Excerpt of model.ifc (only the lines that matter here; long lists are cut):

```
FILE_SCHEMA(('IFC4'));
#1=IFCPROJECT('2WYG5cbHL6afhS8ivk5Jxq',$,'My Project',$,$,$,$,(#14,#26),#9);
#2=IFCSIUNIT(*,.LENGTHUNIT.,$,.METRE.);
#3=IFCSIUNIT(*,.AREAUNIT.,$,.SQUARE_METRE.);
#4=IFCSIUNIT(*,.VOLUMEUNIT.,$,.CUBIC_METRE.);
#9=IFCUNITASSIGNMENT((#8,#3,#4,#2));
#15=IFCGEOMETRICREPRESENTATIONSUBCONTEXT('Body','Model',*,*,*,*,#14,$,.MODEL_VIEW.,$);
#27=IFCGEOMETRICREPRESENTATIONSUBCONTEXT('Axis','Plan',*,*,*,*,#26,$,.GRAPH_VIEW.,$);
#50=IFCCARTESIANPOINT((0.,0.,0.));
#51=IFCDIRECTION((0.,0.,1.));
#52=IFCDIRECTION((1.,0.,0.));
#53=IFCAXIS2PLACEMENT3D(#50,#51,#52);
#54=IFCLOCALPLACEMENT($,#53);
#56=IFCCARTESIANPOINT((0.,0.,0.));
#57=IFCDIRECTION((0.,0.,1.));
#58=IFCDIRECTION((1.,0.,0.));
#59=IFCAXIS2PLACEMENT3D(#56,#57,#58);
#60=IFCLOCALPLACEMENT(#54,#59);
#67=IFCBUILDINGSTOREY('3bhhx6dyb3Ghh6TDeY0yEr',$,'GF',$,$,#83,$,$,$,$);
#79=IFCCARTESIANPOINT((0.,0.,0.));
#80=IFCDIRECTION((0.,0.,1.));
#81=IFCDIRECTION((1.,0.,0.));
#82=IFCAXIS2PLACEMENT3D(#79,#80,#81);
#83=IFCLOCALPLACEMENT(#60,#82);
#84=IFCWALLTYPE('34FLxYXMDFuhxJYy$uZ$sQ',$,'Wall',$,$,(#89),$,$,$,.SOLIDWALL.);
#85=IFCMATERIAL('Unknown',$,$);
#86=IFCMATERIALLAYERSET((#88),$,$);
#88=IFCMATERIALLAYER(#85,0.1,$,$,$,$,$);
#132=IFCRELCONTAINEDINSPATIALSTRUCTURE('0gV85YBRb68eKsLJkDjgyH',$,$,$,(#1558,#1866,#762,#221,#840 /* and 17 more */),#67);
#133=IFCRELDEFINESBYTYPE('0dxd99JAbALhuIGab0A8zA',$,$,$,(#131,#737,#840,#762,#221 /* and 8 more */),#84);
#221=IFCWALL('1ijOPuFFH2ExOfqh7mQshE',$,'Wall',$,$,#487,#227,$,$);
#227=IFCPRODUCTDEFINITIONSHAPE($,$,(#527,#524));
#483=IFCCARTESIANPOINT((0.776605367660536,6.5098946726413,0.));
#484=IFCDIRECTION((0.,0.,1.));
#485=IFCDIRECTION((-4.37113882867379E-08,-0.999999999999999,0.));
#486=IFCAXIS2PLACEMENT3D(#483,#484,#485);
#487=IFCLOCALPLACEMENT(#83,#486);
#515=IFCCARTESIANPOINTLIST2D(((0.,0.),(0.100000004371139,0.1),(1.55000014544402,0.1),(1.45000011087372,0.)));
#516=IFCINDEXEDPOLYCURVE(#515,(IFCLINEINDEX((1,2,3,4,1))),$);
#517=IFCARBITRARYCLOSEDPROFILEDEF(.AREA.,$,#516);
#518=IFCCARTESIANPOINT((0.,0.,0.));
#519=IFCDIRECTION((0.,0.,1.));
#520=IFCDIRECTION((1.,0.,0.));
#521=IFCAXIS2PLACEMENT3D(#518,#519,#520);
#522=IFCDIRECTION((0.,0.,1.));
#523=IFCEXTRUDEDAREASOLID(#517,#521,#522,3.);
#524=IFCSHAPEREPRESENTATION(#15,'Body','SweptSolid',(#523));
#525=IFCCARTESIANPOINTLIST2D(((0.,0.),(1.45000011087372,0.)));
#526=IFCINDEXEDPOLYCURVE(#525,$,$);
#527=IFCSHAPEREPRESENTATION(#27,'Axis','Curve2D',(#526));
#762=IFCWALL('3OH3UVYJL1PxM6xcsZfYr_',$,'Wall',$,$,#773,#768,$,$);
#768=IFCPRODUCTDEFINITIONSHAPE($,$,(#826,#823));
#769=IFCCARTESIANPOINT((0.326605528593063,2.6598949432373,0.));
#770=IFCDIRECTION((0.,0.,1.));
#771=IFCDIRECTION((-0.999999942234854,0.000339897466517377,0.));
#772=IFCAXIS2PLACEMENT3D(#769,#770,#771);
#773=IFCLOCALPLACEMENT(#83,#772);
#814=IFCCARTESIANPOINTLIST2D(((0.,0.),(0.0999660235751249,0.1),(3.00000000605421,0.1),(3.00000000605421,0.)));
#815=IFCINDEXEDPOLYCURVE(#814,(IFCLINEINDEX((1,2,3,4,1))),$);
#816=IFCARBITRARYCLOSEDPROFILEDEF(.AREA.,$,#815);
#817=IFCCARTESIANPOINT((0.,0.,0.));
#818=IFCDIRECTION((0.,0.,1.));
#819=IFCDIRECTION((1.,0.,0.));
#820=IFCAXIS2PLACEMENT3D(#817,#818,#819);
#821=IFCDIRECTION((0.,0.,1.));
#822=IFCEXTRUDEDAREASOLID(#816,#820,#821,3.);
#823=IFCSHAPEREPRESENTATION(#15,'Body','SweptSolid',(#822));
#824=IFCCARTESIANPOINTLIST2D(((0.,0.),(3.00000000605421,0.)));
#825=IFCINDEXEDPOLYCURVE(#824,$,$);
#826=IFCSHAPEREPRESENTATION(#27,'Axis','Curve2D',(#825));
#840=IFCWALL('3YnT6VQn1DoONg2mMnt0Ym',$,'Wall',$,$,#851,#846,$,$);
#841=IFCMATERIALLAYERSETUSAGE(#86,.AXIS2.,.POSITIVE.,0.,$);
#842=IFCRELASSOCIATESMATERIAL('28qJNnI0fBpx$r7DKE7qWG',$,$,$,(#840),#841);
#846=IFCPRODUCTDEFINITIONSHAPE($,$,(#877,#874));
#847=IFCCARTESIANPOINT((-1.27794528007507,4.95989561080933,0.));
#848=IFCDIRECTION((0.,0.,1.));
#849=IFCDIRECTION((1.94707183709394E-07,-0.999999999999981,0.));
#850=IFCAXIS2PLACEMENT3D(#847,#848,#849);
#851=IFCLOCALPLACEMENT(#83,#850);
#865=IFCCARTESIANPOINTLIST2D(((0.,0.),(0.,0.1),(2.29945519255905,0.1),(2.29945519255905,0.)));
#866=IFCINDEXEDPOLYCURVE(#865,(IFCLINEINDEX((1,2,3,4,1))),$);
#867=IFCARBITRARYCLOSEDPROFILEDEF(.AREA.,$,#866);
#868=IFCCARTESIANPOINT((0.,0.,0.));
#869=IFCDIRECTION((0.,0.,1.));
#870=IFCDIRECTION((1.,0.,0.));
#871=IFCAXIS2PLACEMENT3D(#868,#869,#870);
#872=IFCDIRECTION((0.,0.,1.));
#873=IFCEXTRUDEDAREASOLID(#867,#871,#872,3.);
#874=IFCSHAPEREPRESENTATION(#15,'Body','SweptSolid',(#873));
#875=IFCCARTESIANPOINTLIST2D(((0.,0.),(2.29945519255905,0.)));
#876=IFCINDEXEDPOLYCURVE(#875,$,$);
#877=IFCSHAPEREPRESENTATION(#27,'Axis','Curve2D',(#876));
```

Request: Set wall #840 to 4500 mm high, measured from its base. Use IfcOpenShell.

```python
import ifcopenshell
import ifcopenshell.geom
import ifcopenshell.util.representation
import ifcopenshell.util.shape
import ifcopenshell.util.unit

model = ifcopenshell.open("model.ifc")
unit_scale = ifcopenshell.util.unit.calculate_unit_scale(model)
settings = ifcopenshell.geom.settings()


def volume(element):
    """Net volume in cubic metres, openings subtracted."""
    shape = ifcopenshell.geom.create_shape(settings, element)
    return ifcopenshell.util.shape.get_volume(shape.geometry)


wall = model.by_guid("3YnT6VQn1DoONg2mMnt0Ym")
before = volume(wall)

body = ifcopenshell.util.representation.get_representation(wall, "Model", "Body")
solid = body.Items[0]
old_height = solid.Depth
solid.Depth = 4.5 / unit_scale
after = volume(wall)

print(f"height {old_height:g} -> {solid.Depth:g}, volume {before:.3f} -> {after:.3f} m3")

model.write("model-out.ifc")
```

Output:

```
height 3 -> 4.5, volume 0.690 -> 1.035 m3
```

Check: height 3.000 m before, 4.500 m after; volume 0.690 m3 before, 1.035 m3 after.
